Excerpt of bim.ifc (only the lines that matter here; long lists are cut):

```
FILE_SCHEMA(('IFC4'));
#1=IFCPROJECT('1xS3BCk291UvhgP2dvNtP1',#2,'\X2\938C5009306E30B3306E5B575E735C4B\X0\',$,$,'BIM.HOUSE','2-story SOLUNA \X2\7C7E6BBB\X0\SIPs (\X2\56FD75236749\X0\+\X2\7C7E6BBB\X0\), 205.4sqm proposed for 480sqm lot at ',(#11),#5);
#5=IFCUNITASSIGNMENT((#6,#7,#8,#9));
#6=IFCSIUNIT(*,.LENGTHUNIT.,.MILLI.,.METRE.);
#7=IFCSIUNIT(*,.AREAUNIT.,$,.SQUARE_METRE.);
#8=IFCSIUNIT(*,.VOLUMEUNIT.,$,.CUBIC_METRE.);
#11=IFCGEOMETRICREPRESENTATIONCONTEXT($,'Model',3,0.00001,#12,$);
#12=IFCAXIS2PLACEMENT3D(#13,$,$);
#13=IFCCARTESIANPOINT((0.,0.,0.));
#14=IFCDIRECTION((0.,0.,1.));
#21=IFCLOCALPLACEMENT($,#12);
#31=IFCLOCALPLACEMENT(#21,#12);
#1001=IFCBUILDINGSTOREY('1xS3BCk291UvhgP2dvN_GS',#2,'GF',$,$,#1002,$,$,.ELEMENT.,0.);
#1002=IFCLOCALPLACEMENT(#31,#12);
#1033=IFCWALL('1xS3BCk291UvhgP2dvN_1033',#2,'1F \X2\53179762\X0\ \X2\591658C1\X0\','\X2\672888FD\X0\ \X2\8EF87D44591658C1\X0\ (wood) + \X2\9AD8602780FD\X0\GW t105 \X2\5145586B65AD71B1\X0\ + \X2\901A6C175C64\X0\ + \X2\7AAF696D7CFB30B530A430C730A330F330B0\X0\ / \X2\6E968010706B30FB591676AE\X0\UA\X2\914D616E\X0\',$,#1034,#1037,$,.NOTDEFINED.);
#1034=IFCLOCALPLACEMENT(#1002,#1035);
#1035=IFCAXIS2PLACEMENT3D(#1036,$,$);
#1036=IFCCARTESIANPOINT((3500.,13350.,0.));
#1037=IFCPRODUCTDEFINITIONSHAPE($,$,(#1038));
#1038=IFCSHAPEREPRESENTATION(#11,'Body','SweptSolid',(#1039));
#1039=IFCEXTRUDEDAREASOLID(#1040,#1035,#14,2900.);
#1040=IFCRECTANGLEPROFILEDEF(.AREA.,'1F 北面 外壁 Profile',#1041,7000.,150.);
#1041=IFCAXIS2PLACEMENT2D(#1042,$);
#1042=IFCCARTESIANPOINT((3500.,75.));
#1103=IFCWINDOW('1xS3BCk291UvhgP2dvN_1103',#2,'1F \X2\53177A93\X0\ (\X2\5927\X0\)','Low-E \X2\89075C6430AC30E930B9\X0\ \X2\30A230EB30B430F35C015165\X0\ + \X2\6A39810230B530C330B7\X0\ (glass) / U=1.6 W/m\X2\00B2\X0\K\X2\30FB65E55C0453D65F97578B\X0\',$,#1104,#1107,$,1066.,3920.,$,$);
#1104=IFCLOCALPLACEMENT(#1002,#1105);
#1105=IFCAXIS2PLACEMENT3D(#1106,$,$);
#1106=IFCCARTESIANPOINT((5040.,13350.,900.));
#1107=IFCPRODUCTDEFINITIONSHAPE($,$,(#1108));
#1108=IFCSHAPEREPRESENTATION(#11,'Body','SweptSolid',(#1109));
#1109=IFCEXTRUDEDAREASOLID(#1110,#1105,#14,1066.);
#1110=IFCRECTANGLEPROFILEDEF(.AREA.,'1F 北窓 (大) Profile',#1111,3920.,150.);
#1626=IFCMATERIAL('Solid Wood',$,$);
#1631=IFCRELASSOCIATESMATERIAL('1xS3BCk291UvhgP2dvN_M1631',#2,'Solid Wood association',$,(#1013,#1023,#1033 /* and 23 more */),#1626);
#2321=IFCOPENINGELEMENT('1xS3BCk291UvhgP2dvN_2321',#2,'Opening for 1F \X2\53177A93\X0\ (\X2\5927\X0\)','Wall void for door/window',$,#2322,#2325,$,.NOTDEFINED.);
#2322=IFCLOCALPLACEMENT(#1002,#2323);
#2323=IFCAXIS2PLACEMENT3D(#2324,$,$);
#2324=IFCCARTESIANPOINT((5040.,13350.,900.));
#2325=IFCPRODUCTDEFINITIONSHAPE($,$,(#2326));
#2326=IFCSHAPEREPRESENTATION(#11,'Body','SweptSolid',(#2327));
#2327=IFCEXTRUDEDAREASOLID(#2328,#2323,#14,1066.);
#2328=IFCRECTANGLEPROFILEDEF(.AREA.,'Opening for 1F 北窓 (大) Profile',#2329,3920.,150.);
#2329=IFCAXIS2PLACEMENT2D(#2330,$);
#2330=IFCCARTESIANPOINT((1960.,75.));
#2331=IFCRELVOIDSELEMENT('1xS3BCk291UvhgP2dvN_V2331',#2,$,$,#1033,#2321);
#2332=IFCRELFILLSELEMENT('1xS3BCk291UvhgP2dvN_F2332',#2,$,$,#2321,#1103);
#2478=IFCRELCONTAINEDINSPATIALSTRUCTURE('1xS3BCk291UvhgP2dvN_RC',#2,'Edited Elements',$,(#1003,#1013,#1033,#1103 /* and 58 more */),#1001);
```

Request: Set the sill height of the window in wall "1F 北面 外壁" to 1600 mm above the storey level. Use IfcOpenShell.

```python
import numpy as np
import ifcopenshell
import ifcopenshell.api.geometry
import ifcopenshell.geom
import ifcopenshell.util.element
import ifcopenshell.util.placement
import ifcopenshell.util.shape
import ifcopenshell.util.unit

model = ifcopenshell.open("bim.ifc")
unit_scale = ifcopenshell.util.unit.calculate_unit_scale(model)

window = model.by_guid("1xS3BCk291UvhgP2dvN_1103")
opening = window.FillsVoids[0].RelatingOpeningElement
storey = ifcopenshell.util.element.get_container(window, ifc_class="IfcBuildingStorey")
level = ifcopenshell.util.placement.get_local_placement(storey.ObjectPlacement)[2, 3]

# The opening's origin need not be at the sill, so measure its lowest point.
shape = ifcopenshell.geom.create_shape(ifcopenshell.geom.settings(), opening)
bottom = ifcopenshell.util.shape.get_shape_bottom_elevation(shape, shape.geometry) / unit_scale
dz = level + 1.6 / unit_scale - bottom

shift = np.array([0.0, 0.0, dz])
# The window is not placed relative to its opening, so move both.
for product in (opening, window):
    matrix = ifcopenshell.util.placement.get_local_placement(product.ObjectPlacement)
    matrix[:3, 3] += shift
    ifcopenshell.api.geometry.edit_object_placement(model, product=product, matrix=matrix, is_si=False)

print(f"moved by {dz * unit_scale:+.3f} m")

model.write("bim_edited.ifc")
```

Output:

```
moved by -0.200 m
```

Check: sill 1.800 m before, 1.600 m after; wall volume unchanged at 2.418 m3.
